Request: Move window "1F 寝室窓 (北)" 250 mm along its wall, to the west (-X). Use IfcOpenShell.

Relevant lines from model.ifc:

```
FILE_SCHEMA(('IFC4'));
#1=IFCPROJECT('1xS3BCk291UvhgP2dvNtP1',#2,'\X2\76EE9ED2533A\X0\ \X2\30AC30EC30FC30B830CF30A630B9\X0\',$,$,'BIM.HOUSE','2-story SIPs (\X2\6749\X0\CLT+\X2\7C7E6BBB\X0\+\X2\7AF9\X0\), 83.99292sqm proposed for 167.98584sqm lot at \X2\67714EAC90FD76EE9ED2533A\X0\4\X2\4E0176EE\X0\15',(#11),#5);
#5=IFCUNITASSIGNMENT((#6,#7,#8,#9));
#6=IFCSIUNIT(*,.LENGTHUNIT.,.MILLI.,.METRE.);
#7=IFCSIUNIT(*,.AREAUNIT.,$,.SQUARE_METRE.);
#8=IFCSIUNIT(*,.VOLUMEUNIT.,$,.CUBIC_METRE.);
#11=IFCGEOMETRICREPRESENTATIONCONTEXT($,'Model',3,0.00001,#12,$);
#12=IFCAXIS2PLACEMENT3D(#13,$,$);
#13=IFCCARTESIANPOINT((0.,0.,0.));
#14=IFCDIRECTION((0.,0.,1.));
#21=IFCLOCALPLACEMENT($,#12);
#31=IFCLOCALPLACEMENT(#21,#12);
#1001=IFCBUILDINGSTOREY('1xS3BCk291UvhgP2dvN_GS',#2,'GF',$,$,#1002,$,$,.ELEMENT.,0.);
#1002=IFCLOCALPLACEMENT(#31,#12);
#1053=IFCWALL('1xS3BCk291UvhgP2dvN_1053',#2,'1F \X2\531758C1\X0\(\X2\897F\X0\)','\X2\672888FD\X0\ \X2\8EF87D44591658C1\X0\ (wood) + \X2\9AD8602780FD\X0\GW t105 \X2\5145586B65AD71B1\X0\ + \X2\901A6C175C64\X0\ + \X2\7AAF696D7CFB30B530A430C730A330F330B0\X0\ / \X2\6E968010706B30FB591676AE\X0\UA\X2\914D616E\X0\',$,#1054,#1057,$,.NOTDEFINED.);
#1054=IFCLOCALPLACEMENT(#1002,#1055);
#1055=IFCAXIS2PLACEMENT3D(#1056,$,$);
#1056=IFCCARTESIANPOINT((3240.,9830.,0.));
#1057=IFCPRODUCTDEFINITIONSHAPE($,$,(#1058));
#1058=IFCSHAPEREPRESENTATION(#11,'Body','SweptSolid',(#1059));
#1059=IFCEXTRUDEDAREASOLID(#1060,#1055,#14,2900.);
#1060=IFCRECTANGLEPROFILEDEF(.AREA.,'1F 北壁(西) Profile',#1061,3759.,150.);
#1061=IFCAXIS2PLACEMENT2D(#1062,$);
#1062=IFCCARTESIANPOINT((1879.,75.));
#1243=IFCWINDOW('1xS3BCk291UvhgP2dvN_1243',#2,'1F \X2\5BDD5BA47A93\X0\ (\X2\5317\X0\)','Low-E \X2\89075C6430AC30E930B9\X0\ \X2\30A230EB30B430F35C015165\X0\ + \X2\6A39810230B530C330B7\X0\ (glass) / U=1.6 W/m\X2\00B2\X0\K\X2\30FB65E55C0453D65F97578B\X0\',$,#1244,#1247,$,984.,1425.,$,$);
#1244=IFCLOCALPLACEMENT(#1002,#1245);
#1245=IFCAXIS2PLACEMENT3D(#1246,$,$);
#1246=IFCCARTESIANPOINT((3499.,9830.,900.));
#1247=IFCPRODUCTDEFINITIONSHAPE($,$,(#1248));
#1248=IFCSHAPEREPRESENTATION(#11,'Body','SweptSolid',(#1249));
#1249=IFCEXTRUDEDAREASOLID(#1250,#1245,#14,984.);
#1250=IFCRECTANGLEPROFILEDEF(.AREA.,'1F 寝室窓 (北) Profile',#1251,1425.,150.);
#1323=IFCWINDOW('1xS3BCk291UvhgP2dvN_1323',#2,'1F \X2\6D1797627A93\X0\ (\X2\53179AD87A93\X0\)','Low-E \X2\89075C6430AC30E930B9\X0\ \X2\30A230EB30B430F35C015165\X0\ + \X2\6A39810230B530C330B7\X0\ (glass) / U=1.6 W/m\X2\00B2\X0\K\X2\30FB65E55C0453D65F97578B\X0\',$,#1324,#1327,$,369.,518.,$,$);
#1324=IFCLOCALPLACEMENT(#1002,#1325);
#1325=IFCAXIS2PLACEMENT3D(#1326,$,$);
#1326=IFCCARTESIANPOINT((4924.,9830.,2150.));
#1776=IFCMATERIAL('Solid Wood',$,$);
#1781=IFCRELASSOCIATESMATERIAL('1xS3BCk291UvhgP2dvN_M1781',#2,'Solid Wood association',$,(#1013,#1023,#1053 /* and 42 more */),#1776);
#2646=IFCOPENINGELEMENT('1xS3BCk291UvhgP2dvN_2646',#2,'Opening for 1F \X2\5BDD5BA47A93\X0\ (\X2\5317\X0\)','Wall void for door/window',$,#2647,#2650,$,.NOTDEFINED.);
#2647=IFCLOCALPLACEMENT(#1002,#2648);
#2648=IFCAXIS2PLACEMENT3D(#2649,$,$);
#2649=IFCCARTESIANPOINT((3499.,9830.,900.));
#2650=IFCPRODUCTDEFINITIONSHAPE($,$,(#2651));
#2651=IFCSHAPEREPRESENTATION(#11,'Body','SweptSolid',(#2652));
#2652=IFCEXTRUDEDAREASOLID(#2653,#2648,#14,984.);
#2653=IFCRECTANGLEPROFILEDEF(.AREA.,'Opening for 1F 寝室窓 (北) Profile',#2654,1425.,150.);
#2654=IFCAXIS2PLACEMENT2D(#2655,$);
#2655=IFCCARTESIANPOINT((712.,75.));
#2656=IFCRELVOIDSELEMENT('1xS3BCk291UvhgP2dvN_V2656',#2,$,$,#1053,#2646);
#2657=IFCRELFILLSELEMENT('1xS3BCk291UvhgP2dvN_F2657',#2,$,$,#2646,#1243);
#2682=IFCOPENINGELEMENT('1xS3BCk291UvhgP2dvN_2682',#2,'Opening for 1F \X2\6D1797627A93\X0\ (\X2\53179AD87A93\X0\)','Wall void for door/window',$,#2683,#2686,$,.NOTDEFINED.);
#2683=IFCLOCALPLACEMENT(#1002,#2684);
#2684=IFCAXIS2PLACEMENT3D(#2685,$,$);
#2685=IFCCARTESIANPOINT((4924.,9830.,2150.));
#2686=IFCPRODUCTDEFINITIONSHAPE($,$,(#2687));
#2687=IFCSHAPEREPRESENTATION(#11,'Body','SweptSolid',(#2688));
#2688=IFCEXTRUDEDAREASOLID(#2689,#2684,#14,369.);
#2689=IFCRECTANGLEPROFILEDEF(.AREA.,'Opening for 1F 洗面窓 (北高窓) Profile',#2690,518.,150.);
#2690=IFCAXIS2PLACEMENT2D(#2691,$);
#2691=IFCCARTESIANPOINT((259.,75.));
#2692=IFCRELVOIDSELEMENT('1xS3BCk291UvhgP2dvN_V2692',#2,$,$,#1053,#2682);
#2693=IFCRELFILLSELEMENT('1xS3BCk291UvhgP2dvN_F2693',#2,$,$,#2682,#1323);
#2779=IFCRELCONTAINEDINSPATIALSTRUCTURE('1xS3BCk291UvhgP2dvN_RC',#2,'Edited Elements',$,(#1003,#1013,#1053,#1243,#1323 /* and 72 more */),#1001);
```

```python
import ifcopenshell
import ifcopenshell.api.geometry
import ifcopenshell.util.placement

model = ifcopenshell.open("model.ifc")

window = model.by_id(1243)
opening = window.FillsVoids[0].RelatingOpeningElement
wall = opening.VoidsElements[0].RelatingBuildingElement

wall_matrix = ifcopenshell.util.placement.get_local_placement(wall.ObjectPlacement)
shift = wall_matrix[:3, 0] * -250.0
before = ifcopenshell.util.placement.get_local_placement(window.ObjectPlacement)[:3, 3].copy()

# The window is not placed relative to its opening, so move both.
for product in (opening, window):
    matrix = ifcopenshell.util.placement.get_local_placement(product.ObjectPlacement)
    matrix[:3, 3] += shift
    ifcopenshell.api.geometry.edit_object_placement(model, product=product, matrix=matrix, is_si=False)

after = ifcopenshell.util.placement.get_local_placement(window.ObjectPlacement)[:3, 3]
print("window moved by", (after - before).round(3) + 0.0)

model.write("model_rev.ifc")
```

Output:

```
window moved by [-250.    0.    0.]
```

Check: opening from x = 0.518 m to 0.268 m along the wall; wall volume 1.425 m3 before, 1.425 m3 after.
